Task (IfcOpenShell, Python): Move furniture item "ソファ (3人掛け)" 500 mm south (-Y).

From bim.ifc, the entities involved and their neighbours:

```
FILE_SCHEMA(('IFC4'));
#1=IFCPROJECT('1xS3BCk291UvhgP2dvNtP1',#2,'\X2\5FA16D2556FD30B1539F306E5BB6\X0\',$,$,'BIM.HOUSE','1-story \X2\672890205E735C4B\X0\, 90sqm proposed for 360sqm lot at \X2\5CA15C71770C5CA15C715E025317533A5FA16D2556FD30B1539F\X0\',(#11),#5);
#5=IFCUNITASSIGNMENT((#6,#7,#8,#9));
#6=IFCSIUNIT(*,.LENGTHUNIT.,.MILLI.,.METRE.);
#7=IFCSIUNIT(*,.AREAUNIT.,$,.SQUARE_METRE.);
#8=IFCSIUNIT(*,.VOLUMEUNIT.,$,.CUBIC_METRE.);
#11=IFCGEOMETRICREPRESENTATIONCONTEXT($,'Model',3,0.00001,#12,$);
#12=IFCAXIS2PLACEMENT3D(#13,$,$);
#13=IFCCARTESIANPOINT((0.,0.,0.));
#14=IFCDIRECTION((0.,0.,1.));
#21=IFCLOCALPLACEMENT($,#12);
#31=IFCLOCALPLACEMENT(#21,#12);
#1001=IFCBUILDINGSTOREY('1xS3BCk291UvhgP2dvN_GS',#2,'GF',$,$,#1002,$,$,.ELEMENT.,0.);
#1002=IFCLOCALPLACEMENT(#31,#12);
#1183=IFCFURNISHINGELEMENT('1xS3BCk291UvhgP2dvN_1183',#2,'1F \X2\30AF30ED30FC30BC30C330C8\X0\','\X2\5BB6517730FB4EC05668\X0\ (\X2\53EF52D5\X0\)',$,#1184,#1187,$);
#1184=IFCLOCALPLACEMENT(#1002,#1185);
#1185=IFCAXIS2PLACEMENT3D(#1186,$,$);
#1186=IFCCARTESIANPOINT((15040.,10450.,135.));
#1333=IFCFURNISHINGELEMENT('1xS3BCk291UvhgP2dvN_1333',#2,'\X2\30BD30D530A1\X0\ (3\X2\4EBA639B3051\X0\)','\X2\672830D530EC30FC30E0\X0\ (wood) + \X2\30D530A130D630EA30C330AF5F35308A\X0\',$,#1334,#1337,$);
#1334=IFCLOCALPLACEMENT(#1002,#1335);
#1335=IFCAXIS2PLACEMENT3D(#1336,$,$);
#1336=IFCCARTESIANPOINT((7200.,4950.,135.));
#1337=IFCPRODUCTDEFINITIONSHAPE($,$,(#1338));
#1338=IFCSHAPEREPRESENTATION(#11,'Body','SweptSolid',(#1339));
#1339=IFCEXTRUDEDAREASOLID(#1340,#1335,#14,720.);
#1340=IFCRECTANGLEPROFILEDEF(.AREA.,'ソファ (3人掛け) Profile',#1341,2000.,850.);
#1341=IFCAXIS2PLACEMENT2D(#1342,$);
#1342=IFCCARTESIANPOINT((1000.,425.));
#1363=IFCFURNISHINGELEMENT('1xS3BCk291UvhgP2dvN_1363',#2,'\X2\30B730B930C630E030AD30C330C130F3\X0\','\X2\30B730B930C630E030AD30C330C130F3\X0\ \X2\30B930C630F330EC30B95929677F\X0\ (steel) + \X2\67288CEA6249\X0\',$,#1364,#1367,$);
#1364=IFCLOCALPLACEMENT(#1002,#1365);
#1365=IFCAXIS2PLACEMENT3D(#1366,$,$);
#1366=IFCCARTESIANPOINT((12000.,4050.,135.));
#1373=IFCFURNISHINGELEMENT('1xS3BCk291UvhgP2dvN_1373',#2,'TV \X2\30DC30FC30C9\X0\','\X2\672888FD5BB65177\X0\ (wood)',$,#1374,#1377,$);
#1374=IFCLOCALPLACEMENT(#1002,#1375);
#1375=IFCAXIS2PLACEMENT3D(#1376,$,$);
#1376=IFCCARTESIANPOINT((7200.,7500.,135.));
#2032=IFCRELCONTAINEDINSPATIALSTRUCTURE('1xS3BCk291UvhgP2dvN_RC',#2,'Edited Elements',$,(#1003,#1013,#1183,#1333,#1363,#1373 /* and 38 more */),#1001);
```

```python
import ifcopenshell
import ifcopenshell.api.geometry
import ifcopenshell.util.placement
import ifcopenshell.util.unit

model = ifcopenshell.open("bim.ifc")
unit_scale = ifcopenshell.util.unit.calculate_unit_scale(model)

item = model.by_id(1333)
matrix = ifcopenshell.util.placement.get_local_placement(item.ObjectPlacement)
matrix[1, 3] -= 0.5 / unit_scale
ifcopenshell.api.geometry.edit_object_placement(model, product=item, matrix=matrix, is_si=False)

print(ifcopenshell.util.placement.get_local_placement(item.ObjectPlacement).round(3) + 0.0)

model.write("bim_updated.ifc")
```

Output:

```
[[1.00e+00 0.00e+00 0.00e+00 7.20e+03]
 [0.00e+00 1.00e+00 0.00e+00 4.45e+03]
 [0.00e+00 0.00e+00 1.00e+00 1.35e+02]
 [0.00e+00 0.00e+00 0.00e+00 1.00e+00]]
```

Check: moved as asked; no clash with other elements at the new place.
